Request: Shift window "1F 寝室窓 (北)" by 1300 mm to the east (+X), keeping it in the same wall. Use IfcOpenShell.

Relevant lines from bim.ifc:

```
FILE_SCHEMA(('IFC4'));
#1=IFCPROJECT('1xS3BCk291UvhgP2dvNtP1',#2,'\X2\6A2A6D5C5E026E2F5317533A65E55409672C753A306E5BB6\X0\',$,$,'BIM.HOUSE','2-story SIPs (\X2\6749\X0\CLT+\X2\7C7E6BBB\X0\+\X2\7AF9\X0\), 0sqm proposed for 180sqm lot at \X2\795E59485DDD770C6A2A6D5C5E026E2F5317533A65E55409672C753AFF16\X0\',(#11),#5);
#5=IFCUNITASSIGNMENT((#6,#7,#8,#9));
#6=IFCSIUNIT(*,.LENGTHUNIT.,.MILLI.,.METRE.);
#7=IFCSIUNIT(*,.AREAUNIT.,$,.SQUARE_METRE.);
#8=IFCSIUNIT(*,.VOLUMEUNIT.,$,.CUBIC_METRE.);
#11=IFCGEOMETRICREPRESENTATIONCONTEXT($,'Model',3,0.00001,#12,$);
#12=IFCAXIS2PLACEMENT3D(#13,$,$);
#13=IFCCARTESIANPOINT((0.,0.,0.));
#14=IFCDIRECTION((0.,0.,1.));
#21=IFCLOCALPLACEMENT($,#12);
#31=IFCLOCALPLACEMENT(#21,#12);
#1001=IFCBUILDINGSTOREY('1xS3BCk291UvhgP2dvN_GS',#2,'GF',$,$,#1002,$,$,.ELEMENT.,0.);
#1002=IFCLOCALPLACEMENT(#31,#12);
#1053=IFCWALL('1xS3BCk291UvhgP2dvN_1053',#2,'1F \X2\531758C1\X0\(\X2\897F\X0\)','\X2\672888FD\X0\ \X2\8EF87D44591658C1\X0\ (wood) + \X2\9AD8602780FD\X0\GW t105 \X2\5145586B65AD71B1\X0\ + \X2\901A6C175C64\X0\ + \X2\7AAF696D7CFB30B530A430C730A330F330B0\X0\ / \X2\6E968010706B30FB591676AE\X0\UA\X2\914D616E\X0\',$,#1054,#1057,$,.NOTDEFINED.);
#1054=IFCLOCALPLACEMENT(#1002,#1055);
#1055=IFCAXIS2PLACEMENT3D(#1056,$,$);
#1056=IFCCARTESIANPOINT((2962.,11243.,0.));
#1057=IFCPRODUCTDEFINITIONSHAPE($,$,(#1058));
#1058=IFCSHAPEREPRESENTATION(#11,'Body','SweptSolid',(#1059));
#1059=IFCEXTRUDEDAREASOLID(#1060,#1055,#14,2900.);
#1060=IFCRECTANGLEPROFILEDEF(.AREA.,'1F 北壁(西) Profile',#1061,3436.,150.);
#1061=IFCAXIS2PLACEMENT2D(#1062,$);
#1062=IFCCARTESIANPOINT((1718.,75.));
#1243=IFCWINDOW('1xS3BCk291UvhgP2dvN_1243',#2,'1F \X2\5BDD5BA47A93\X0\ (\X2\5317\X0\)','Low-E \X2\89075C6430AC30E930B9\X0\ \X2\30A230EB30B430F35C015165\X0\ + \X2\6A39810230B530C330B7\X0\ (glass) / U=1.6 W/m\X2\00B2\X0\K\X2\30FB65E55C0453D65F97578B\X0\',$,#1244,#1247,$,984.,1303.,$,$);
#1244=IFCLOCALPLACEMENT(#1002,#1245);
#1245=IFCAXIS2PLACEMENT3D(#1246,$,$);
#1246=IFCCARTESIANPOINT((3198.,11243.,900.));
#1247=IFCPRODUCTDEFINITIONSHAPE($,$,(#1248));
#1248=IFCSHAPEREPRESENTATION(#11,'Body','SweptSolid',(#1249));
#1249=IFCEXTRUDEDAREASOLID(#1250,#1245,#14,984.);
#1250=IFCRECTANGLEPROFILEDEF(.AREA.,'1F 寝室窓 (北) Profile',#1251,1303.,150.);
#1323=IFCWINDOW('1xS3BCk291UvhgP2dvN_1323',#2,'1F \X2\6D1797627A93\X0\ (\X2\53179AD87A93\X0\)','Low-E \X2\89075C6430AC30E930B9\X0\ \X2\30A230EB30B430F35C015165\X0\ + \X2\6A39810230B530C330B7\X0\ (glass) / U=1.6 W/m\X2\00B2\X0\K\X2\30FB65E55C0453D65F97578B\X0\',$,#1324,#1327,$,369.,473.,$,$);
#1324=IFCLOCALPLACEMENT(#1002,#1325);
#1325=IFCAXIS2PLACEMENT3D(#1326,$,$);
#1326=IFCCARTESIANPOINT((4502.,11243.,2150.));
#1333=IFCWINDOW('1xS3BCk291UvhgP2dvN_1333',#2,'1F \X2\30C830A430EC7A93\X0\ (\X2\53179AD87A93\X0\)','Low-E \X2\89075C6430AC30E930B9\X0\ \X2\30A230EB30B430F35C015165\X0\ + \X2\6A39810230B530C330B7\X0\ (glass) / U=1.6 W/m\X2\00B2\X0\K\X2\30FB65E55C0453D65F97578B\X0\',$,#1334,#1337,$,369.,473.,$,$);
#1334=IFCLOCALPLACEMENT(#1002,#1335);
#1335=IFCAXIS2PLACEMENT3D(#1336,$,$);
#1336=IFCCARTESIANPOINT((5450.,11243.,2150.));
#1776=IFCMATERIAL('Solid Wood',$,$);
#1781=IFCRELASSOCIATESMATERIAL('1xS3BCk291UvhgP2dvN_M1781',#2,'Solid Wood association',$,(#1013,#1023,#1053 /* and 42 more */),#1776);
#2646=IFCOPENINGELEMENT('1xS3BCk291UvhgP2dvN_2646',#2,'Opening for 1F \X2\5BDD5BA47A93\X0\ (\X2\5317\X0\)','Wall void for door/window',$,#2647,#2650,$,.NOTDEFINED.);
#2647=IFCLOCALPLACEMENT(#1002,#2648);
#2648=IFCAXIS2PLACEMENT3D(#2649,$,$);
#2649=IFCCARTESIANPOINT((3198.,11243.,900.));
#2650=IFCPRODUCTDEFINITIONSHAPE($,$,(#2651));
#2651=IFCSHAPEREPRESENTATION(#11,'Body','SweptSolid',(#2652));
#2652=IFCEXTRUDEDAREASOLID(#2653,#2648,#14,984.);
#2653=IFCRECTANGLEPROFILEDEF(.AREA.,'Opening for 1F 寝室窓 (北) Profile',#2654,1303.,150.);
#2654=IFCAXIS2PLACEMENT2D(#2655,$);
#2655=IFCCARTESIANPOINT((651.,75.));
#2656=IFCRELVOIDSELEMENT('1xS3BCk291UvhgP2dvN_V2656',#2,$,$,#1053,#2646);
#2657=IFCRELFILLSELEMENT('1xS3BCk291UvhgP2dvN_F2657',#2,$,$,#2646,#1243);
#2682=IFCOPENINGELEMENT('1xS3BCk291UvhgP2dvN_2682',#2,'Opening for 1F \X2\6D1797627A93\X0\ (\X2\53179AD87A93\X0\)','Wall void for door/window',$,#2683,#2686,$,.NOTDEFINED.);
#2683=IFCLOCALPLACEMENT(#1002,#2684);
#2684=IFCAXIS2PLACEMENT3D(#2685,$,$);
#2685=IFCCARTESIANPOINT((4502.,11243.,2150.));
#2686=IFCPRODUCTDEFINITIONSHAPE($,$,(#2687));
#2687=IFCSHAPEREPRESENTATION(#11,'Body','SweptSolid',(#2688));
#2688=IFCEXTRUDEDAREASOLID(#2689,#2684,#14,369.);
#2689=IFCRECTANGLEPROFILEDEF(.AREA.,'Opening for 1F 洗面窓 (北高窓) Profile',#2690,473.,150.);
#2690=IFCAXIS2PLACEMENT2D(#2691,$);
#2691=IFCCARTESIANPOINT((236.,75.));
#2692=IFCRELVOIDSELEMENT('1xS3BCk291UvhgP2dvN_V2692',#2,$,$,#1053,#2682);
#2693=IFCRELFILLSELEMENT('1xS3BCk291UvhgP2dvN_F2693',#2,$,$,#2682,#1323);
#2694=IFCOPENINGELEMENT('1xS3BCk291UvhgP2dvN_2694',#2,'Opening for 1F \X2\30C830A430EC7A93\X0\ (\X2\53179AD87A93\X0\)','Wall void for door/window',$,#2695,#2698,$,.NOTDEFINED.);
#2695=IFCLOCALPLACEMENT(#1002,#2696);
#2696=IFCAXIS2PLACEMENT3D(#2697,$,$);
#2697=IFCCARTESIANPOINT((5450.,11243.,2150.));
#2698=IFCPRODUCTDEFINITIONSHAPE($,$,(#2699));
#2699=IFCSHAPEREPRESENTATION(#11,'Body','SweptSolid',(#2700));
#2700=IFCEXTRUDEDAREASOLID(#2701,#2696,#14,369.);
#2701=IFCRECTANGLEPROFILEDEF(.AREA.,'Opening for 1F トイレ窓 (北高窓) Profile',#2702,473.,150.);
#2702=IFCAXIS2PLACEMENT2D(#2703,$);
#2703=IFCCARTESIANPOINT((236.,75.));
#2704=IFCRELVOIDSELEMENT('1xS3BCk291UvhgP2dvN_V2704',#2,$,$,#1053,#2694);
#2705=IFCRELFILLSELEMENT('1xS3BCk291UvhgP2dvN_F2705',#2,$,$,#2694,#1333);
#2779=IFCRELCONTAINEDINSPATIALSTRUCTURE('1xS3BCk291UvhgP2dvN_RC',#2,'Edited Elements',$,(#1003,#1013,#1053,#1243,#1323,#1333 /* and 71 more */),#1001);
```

```python
import ifcopenshell
import ifcopenshell.api.geometry
import ifcopenshell.util.placement
import ifcopenshell.util.unit

model = ifcopenshell.open("bim.ifc")
unit_scale = ifcopenshell.util.unit.calculate_unit_scale(model)

window = model.by_guid("1xS3BCk291UvhgP2dvN_1243")
opening = window.FillsVoids[0].RelatingOpeningElement
wall = opening.VoidsElements[0].RelatingBuildingElement

wall_matrix = ifcopenshell.util.placement.get_local_placement(wall.ObjectPlacement)
shift = wall_matrix[:3, 0] * 1.3 / unit_scale
before = ifcopenshell.util.placement.get_local_placement(window.ObjectPlacement)[:3, 3].copy()

# The window is not placed relative to its opening, so move both.
for product in (opening, window):
    matrix = ifcopenshell.util.placement.get_local_placement(product.ObjectPlacement)
    matrix[:3, 3] += shift
    ifcopenshell.api.geometry.edit_object_placement(model, product=product, matrix=matrix, is_si=False)

after = ifcopenshell.util.placement.get_local_placement(window.ObjectPlacement)[:3, 3]
print("window moved by", (after - before).round(3) + 0.0)

model.write("bim_edited.ifc")
```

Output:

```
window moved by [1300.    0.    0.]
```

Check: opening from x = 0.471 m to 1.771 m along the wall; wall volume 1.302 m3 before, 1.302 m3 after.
